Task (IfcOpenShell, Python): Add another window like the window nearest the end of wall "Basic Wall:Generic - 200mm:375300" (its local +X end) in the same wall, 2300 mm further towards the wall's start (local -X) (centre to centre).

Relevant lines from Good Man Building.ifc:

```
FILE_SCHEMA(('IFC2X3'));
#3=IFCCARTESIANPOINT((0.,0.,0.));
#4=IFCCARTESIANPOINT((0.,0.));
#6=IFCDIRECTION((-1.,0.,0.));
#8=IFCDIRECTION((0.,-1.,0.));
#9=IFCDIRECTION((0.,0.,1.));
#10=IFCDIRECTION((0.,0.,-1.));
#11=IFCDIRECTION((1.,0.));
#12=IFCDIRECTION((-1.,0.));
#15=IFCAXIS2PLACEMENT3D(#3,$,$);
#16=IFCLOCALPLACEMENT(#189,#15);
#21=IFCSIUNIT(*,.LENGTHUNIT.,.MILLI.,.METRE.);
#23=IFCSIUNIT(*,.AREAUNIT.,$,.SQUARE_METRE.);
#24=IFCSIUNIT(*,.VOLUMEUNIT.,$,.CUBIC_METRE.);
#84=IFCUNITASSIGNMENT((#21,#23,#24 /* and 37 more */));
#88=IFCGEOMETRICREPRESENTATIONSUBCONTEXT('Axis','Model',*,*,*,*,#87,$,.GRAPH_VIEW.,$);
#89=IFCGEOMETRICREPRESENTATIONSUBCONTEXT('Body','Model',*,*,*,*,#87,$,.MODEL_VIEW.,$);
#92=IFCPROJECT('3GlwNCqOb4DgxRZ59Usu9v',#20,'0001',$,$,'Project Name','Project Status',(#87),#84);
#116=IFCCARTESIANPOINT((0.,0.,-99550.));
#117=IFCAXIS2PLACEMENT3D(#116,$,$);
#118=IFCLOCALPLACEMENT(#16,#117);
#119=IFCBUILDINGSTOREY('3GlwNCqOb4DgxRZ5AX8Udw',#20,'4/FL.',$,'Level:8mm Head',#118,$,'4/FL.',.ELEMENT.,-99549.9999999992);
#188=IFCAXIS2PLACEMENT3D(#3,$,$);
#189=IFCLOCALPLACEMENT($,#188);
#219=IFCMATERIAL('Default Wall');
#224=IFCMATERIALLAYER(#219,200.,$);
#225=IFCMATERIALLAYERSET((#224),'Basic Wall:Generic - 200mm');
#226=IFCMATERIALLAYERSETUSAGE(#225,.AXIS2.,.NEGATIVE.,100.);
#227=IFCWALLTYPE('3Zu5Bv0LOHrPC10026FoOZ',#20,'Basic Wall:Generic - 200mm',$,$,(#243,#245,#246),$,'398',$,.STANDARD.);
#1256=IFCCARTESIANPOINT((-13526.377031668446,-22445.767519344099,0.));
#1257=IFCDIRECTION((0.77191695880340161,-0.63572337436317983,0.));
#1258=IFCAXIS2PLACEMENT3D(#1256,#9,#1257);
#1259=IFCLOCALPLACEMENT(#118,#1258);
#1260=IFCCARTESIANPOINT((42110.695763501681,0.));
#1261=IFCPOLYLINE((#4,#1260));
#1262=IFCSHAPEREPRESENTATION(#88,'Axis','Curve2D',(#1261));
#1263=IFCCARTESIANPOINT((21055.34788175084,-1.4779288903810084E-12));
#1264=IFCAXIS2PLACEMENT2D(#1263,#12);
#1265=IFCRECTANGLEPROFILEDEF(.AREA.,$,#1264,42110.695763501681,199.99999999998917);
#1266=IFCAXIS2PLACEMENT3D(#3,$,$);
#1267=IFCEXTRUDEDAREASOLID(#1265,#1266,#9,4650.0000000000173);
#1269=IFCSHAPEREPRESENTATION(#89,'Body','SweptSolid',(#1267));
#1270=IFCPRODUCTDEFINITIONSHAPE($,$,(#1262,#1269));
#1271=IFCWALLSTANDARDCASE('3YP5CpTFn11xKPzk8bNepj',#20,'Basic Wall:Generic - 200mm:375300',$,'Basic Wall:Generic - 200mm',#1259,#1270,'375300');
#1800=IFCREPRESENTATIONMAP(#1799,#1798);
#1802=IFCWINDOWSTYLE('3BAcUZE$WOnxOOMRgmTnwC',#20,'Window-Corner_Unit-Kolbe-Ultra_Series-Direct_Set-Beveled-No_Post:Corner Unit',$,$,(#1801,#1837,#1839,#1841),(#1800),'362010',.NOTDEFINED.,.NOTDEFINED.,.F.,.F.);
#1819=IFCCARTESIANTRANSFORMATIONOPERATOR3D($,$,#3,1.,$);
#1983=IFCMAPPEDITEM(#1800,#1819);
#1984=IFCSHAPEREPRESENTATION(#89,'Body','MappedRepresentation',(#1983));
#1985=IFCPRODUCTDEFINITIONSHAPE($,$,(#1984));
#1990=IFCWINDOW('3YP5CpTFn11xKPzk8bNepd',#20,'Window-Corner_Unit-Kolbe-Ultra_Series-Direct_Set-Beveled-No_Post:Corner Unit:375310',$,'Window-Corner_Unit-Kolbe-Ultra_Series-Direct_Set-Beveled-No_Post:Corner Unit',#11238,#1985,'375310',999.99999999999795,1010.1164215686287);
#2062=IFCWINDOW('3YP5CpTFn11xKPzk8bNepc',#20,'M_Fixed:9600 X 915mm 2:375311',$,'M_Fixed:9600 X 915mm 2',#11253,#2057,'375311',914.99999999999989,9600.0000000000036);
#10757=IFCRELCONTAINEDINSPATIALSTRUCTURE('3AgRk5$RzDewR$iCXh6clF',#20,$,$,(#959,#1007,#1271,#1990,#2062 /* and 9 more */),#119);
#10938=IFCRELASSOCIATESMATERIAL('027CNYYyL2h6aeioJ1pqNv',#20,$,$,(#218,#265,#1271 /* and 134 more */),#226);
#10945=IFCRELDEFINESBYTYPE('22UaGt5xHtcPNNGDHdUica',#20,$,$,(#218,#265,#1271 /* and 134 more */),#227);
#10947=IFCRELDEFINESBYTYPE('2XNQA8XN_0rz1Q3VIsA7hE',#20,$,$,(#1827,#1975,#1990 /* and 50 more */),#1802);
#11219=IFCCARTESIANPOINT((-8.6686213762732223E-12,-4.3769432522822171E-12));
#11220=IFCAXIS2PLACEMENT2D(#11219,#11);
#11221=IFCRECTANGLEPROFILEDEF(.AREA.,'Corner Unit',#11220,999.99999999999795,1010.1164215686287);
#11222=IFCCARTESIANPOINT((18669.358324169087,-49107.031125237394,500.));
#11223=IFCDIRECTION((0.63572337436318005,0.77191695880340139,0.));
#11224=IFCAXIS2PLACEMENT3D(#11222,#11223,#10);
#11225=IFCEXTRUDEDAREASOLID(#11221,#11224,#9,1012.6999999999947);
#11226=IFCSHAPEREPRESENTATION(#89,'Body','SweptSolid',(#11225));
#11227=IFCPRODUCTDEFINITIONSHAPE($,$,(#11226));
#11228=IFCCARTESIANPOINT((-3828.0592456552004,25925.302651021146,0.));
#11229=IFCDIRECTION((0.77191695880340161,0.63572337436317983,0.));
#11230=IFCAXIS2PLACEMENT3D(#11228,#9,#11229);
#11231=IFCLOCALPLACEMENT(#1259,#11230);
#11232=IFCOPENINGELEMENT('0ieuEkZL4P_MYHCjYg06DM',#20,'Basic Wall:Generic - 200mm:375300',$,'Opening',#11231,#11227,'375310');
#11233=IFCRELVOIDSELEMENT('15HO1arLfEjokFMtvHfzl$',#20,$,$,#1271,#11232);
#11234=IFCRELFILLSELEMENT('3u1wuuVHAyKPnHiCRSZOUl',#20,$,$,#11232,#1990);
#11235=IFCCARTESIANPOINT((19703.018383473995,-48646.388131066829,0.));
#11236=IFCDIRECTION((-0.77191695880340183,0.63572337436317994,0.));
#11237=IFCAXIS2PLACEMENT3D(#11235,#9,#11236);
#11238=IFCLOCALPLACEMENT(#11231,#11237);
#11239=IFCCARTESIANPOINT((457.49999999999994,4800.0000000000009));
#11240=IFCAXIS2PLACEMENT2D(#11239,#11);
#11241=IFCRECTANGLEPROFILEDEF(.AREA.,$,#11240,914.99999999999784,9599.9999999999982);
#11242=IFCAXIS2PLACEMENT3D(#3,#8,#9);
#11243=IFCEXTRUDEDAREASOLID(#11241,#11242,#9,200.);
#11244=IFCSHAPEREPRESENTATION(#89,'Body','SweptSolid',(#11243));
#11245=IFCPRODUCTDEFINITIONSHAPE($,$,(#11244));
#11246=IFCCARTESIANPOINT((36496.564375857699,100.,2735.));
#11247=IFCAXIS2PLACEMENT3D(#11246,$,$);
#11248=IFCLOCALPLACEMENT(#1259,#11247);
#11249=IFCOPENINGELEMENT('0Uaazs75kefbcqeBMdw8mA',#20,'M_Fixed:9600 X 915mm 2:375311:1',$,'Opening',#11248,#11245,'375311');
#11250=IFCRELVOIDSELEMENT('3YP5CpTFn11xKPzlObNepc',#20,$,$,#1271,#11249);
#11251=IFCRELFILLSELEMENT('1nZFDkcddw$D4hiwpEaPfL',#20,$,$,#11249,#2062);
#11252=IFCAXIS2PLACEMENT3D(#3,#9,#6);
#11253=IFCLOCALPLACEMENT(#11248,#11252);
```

```python
import ifcopenshell
import ifcopenshell.api.feature
import ifcopenshell.api.geometry
import ifcopenshell.api.root
import ifcopenshell.geom
import ifcopenshell.util.element
import ifcopenshell.util.placement
import ifcopenshell.util.shape

model = ifcopenshell.open("Good Man Building.ifc")
settings = ifcopenshell.geom.settings()


def volume(element):
    """Net volume in cubic metres, openings subtracted."""
    shape = ifcopenshell.geom.create_shape(settings, element)
    return ifcopenshell.util.shape.get_volume(shape.geometry)


def reuse_history(source, copy):
    """copy_class also copies each property set's owner history, people and application; keep the originals."""
    for rel in copy.IsDefinedBy:
        if rel.is_a("IfcRelDefinesByProperties") and (history := rel.RelatingPropertyDefinition.OwnerHistory):
            rel.RelatingPropertyDefinition.OwnerHistory = source.OwnerHistory
            ifcopenshell.util.element.remove_deep2(model, history)


window = model.by_guid("3YP5CpTFn11xKPzk8bNepd")
opening = window.FillsVoids[0].RelatingOpeningElement
wall = opening.VoidsElements[0].RelatingBuildingElement
before = volume(wall)
shift = ifcopenshell.util.placement.get_local_placement(wall.ObjectPlacement)[:3, 0] * -2300.0

# copy_class copies the void relationship, type, container and properties, but no geometry.
new_opening = ifcopenshell.api.root.copy_class(model, product=opening)
new_opening.Representation = ifcopenshell.util.element.copy_deep(
    model, opening.Representation, exclude=["IfcGeometricRepresentationContext", "IfcRepresentationMap"]
)
new_opening.Name = "Basic Wall:Generic - 200mm"
new_opening.Tag = None
new_window = ifcopenshell.api.root.copy_class(model, product=window)
new_window.Representation = ifcopenshell.util.element.copy_deep(
    model, window.Representation, exclude=["IfcGeometricRepresentationContext", "IfcRepresentationMap"]
)
new_window.Name = "Window-Corner_Unit-Kolbe-Ultra_Series-Direct_Set-Beveled-No_Post:Corner Unit"
new_window.Tag = None
reuse_history(window, new_window)
fills = ifcopenshell.api.feature.add_filling(model, opening=new_opening, element=new_window)
fills.OwnerHistory = new_window.OwnerHistory  # required in IFC2X3

for old, new in ((opening, new_opening), (window, new_window)):
    matrix = ifcopenshell.util.placement.get_local_placement(old.ObjectPlacement)
    matrix[:3, 3] += shift
    ifcopenshell.api.geometry.edit_object_placement(model, product=new, matrix=matrix, is_si=False)

after = volume(wall)

print(f"wall volume {before:.3f} -> {after:.3f} m3")

model.write("Good Man Building_edited.ifc")
```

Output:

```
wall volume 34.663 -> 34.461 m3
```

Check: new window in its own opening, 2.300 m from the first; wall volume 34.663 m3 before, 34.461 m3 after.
